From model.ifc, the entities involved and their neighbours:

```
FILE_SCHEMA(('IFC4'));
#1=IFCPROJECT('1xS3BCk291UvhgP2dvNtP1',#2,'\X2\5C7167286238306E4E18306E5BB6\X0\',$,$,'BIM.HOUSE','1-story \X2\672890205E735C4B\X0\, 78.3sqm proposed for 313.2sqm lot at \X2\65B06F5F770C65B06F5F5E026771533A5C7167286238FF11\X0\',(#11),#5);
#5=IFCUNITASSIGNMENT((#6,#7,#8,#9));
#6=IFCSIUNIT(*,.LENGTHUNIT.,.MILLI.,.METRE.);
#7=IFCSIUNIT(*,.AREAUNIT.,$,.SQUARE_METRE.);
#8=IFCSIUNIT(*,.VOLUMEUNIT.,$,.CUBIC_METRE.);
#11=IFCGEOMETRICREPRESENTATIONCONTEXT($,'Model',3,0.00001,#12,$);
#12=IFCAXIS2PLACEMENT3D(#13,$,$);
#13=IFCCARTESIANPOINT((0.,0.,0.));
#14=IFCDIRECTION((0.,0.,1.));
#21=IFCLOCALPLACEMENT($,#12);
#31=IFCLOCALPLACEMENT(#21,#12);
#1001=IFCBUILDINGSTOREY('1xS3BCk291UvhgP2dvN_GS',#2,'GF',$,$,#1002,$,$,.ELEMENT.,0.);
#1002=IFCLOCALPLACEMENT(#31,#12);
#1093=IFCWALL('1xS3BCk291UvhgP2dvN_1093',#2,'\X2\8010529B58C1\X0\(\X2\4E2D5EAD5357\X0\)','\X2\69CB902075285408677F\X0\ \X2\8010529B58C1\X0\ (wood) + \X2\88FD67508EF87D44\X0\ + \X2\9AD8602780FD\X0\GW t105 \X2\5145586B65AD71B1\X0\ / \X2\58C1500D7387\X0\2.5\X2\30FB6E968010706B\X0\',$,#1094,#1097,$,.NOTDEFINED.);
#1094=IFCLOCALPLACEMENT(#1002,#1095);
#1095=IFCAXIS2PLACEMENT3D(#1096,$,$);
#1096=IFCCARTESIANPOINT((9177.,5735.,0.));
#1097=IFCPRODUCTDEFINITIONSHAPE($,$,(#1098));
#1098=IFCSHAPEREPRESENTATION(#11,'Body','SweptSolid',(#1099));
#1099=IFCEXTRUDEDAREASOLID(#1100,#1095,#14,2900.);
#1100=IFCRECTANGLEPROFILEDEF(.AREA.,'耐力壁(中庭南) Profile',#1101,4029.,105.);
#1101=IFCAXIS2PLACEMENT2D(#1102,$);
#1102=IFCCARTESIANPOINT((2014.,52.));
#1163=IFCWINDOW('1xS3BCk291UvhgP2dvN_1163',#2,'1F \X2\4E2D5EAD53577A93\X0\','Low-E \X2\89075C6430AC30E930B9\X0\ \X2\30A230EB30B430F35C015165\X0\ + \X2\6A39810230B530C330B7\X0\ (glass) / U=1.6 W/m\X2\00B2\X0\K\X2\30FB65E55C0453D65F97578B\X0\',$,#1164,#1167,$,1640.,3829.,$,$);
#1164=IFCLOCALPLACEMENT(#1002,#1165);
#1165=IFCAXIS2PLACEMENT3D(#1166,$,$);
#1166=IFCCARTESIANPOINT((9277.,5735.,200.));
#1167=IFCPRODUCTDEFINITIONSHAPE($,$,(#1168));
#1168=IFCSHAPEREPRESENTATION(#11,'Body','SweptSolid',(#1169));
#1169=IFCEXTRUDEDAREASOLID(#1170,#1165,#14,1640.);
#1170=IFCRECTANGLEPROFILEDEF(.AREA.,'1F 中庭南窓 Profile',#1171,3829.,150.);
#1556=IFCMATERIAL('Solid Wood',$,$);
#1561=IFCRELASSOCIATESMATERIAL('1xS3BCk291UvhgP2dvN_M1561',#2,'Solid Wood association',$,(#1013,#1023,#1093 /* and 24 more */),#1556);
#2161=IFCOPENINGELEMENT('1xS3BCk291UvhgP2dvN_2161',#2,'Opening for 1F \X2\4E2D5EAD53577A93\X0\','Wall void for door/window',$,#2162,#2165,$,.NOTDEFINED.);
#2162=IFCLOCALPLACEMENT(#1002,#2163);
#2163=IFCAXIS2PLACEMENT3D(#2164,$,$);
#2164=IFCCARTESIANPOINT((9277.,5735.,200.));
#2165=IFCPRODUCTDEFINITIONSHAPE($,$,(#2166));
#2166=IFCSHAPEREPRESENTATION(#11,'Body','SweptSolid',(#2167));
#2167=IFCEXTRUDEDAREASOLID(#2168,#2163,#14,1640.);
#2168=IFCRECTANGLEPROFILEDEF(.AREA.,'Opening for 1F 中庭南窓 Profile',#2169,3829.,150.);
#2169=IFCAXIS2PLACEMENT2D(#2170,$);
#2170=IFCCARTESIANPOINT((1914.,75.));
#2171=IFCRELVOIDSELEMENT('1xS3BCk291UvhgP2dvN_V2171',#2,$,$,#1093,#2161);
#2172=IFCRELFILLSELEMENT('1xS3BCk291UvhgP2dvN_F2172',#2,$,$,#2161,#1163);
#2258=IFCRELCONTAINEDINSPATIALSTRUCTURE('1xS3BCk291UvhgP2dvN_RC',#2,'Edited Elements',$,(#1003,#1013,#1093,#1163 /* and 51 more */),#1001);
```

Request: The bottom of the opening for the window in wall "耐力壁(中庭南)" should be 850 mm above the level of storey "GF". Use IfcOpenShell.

```python
import numpy as np
import ifcopenshell
import ifcopenshell.api.geometry
import ifcopenshell.geom
import ifcopenshell.util.element
import ifcopenshell.util.placement
import ifcopenshell.util.shape
import ifcopenshell.util.unit

model = ifcopenshell.open("model.ifc")
unit_scale = ifcopenshell.util.unit.calculate_unit_scale(model)

window = model.by_guid("1xS3BCk291UvhgP2dvN_1163")
opening = window.FillsVoids[0].RelatingOpeningElement
storey = ifcopenshell.util.element.get_container(window, ifc_class="IfcBuildingStorey")
level = ifcopenshell.util.placement.get_local_placement(storey.ObjectPlacement)[2, 3]

# The opening's origin need not be at the sill, so measure its lowest point.
shape = ifcopenshell.geom.create_shape(ifcopenshell.geom.settings(), opening)
bottom = ifcopenshell.util.shape.get_shape_bottom_elevation(shape, shape.geometry) / unit_scale
dz = level + 850.0 - bottom

shift = np.array([0.0, 0.0, dz])
# The window is not placed relative to its opening, so move both.
for product in (opening, window):
    matrix = ifcopenshell.util.placement.get_local_placement(product.ObjectPlacement)
    matrix[:3, 3] += shift
    ifcopenshell.api.geometry.edit_object_placement(model, product=product, matrix=matrix, is_si=False)

print(f"moved by {dz * unit_scale:+.3f} m")

model.write("model_updated.ifc")
```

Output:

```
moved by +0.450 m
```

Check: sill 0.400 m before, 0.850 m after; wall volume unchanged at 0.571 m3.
